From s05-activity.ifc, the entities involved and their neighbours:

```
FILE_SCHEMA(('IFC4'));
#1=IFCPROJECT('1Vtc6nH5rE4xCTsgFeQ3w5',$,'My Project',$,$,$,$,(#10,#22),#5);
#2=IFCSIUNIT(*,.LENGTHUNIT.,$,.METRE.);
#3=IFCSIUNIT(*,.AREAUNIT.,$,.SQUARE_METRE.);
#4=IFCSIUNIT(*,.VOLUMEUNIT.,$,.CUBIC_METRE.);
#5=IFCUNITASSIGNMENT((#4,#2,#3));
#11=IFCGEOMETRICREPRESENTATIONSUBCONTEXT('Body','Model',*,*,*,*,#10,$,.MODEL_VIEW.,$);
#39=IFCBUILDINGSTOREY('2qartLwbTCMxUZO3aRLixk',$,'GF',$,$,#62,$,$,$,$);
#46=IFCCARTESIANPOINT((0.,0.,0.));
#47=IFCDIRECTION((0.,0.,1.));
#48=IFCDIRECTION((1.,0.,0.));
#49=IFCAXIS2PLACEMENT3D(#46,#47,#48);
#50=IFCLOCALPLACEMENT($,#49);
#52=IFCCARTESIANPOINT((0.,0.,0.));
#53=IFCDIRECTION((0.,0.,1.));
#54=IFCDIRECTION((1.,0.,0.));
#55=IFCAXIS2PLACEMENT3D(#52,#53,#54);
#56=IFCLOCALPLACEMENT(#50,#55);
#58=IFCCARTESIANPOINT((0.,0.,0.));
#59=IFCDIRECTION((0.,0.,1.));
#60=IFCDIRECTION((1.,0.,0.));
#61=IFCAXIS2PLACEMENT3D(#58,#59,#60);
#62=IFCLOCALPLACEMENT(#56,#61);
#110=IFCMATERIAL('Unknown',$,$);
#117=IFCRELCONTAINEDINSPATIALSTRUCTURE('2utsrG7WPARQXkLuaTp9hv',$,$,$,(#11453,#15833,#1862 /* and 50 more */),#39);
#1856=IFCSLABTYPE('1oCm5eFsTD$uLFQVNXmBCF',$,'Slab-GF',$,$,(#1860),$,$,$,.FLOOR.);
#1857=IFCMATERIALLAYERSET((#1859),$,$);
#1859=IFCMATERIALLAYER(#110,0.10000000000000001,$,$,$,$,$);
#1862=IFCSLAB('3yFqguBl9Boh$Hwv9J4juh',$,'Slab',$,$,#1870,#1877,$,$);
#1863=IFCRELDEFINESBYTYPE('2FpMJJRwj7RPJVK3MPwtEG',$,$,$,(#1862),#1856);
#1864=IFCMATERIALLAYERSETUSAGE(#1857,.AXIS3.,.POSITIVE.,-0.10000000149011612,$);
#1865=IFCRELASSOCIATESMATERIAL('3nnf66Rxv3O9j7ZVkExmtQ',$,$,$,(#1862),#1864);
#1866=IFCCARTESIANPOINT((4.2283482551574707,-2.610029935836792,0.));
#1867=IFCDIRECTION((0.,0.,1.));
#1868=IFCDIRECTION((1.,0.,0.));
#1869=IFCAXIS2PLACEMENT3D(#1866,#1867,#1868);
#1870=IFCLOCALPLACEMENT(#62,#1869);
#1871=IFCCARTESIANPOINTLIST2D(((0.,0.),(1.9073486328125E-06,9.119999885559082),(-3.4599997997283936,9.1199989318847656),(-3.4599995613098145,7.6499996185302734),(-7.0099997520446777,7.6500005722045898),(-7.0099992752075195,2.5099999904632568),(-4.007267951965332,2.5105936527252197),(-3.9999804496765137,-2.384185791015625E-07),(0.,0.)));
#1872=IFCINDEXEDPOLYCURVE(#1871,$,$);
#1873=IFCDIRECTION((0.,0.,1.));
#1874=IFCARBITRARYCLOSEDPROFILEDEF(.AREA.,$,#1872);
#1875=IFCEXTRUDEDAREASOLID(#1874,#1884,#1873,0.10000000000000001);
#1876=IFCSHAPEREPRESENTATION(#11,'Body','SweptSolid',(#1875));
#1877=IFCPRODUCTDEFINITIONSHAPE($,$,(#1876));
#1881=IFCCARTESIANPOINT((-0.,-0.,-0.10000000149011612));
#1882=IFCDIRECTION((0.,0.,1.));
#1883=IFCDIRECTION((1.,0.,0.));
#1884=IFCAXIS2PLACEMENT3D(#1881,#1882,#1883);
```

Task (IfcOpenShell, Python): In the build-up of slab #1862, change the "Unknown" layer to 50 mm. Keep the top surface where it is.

```python
import ifcopenshell
import ifcopenshell.util.element
import ifcopenshell.util.representation
import ifcopenshell.util.unit

model = ifcopenshell.open("s05-activity.ifc")
unit_scale = ifcopenshell.util.unit.calculate_unit_scale(model)

layer_set = model.by_id(1857)
layer = next(l for l in layer_set.MaterialLayers if l.Material and l.Material.Name == "Unknown")
change = 0.05 / unit_scale - layer.LayerThickness
layer.LayerThickness += change

# Geometry does not follow the layer set by itself.
slabs = [e for e in ifcopenshell.util.element.get_elements_by_material(model, layer_set) if e.is_a("IfcSlab")]
for slab in sorted(slabs, key=lambda e: e.id()):
    body = ifcopenshell.util.representation.get_representation(slab, "Model", "Body")
    solid = body.Items[0]
    old_depth = solid.Depth
    solid.Depth += change
    # Extruded upwards: lower the start of the extrusion so the top stays.
    x, y, z = solid.Position.Location.Coordinates
    solid.Position.Location = model.createIfcCartesianPoint((x, y, z - change))
    print(slab.id(), f"{old_depth:g} -> {solid.Depth:g}")

# The layers are counted up from the underside, which has moved.
for usage in {ifcopenshell.util.element.get_material(slab) for slab in slabs}:
    usage.OffsetFromReferenceLine -= change

model.write("s05-activity_v2.ifc")
```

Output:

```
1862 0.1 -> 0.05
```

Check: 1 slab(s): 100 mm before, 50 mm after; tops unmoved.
